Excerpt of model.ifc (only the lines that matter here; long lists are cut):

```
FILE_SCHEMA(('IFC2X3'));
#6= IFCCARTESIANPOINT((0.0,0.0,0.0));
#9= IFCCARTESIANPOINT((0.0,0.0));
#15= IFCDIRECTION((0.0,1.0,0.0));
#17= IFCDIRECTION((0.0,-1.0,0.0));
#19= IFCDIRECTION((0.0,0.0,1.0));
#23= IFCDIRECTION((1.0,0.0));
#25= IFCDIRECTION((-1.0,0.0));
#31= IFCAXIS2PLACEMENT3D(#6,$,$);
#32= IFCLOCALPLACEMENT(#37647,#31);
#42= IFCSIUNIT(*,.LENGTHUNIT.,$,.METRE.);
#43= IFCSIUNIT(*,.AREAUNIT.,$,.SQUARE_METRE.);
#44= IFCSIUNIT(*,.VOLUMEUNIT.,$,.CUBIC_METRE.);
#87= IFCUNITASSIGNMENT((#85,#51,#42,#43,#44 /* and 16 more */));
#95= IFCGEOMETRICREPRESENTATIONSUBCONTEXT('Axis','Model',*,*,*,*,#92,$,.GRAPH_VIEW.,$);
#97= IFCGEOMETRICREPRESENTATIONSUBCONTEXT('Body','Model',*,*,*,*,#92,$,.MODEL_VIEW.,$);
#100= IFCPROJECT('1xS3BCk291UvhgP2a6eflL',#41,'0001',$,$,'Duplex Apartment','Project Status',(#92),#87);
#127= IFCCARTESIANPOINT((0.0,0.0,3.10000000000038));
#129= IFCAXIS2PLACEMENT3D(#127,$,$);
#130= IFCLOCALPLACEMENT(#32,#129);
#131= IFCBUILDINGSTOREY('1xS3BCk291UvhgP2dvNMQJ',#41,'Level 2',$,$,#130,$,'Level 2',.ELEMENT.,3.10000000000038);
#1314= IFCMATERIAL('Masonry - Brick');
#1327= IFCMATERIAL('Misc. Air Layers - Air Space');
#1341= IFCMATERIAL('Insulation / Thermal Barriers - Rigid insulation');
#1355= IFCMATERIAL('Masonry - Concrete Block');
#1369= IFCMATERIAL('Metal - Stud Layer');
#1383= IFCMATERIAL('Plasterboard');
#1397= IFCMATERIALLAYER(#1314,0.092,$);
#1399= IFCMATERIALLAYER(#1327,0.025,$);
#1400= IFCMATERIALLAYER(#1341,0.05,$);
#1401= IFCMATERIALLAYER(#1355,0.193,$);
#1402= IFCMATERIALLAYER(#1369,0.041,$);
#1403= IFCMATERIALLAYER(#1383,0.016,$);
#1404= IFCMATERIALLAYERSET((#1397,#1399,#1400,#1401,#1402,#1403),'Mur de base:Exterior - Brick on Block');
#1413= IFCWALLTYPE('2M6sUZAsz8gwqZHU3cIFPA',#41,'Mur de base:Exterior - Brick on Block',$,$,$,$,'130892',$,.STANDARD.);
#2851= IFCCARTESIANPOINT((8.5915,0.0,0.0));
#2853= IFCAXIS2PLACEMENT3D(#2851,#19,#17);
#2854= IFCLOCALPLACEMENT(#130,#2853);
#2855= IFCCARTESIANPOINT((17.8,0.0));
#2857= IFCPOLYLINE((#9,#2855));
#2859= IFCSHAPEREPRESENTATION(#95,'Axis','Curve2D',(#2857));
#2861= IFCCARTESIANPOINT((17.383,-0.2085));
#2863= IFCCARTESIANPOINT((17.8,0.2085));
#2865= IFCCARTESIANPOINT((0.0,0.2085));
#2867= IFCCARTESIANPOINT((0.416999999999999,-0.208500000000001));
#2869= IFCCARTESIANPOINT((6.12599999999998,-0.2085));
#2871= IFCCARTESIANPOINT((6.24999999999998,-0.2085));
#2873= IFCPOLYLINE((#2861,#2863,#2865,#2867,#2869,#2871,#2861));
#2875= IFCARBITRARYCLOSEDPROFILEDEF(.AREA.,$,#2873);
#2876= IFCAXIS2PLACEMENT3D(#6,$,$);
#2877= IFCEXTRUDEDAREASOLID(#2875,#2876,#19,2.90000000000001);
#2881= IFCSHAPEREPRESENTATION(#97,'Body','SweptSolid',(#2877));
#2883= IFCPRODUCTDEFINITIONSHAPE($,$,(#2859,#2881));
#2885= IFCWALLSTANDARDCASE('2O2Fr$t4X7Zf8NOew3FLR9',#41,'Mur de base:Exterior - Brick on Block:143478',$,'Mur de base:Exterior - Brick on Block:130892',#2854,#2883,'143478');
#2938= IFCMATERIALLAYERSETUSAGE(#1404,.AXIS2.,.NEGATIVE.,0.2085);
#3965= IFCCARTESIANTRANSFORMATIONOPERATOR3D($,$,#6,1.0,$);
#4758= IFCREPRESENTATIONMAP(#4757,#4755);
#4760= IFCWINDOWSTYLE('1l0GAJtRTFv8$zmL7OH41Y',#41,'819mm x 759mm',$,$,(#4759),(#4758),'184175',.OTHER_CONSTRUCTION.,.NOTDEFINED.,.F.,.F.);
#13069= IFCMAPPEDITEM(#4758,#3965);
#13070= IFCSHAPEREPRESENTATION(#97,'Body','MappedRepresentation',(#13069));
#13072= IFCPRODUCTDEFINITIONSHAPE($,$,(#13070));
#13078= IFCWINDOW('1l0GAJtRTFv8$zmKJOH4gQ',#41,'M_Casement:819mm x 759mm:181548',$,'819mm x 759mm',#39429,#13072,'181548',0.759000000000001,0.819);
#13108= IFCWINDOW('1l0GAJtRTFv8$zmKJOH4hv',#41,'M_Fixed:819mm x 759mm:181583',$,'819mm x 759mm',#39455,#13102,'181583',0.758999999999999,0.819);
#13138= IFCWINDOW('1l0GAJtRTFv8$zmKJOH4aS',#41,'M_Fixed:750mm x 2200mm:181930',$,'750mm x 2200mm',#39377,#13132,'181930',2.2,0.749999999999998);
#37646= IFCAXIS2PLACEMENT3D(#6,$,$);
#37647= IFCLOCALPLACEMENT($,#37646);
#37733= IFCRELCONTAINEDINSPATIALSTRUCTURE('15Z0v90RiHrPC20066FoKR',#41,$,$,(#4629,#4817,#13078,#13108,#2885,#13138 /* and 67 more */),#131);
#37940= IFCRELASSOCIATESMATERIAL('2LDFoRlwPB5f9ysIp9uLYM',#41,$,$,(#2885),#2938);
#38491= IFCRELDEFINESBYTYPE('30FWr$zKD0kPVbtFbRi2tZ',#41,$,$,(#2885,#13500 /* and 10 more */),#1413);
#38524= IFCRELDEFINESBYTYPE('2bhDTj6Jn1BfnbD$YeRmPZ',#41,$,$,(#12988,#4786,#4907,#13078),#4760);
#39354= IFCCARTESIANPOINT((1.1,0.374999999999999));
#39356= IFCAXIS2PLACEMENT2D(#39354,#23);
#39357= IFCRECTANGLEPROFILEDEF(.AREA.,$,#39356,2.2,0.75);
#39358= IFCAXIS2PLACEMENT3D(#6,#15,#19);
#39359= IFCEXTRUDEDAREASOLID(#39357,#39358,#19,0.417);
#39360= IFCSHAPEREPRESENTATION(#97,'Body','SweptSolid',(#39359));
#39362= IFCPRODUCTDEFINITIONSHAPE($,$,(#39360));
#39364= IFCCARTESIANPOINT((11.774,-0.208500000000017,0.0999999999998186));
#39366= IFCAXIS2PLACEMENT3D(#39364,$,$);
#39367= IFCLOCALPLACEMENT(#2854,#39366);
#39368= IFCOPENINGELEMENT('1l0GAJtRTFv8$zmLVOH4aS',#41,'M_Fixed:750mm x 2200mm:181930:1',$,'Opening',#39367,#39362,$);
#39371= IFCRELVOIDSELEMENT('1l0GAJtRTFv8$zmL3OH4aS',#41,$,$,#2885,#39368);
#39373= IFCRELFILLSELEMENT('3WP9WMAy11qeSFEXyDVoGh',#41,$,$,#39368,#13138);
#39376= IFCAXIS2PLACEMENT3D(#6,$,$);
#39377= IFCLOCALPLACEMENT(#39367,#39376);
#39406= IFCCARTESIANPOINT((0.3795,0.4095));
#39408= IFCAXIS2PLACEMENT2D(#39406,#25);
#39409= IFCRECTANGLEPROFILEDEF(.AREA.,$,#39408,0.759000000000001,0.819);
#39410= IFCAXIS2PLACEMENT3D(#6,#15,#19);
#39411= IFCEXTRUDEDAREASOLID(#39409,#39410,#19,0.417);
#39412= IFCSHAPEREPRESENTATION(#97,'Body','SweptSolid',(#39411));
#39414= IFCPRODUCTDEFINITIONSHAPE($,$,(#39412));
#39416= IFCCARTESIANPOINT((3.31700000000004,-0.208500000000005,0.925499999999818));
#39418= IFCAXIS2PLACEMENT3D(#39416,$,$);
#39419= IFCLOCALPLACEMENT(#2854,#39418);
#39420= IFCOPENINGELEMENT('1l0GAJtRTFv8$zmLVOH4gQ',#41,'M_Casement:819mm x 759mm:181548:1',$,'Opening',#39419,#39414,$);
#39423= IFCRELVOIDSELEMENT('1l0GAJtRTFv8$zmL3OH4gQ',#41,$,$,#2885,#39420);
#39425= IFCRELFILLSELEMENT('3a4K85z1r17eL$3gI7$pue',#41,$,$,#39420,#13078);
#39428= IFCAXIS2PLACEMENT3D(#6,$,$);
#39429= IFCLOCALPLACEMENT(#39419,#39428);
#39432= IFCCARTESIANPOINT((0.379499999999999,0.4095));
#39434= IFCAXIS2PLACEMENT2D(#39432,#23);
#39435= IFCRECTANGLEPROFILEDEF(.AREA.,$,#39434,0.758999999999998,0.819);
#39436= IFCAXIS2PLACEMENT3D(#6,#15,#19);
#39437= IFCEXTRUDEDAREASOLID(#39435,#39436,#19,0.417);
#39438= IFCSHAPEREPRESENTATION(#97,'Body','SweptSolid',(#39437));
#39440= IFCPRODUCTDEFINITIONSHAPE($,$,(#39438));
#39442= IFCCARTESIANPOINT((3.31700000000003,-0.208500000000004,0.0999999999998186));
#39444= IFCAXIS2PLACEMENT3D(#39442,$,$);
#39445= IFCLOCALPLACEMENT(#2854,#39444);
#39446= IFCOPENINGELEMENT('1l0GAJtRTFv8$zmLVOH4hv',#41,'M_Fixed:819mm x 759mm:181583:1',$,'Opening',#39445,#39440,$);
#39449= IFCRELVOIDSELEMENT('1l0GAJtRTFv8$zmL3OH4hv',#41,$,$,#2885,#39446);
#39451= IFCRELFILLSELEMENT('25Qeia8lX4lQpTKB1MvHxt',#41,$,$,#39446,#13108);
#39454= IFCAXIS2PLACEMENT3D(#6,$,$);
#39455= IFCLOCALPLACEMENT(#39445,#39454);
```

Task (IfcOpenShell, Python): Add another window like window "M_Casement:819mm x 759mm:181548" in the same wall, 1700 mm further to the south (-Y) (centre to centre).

```python
import ifcopenshell
import ifcopenshell.api.feature
import ifcopenshell.api.geometry
import ifcopenshell.api.root
import ifcopenshell.geom
import ifcopenshell.util.element
import ifcopenshell.util.placement
import ifcopenshell.util.shape
import ifcopenshell.util.unit

model = ifcopenshell.open("model.ifc")
unit_scale = ifcopenshell.util.unit.calculate_unit_scale(model)
settings = ifcopenshell.geom.settings()


def volume(element):
    """Net volume in cubic metres, openings subtracted."""
    shape = ifcopenshell.geom.create_shape(settings, element)
    return ifcopenshell.util.shape.get_volume(shape.geometry)


def reuse_history(source, copy):
    """copy_class also copies each property set's owner history, people and application; keep the originals."""
    for rel in copy.IsDefinedBy:
        if rel.is_a("IfcRelDefinesByProperties") and (history := rel.RelatingPropertyDefinition.OwnerHistory):
            rel.RelatingPropertyDefinition.OwnerHistory = source.OwnerHistory
            ifcopenshell.util.element.remove_deep2(model, history)


window = model.by_guid("1l0GAJtRTFv8$zmKJOH4gQ")
opening = window.FillsVoids[0].RelatingOpeningElement
wall = opening.VoidsElements[0].RelatingBuildingElement
before = volume(wall)
shift = ifcopenshell.util.placement.get_local_placement(wall.ObjectPlacement)[:3, 0] * 1.7 / unit_scale

# copy_class copies the void relationship, type, container and properties, but no geometry.
new_opening = ifcopenshell.api.root.copy_class(model, product=opening)
new_opening.Representation = ifcopenshell.util.element.copy_deep(
    model, opening.Representation, exclude=["IfcGeometricRepresentationContext", "IfcRepresentationMap"]
)
new_opening.Name = "M_Casement:819mm x 759mm"
new_window = ifcopenshell.api.root.copy_class(model, product=window)
new_window.Representation = ifcopenshell.util.element.copy_deep(
    model, window.Representation, exclude=["IfcGeometricRepresentationContext", "IfcRepresentationMap"]
)
new_window.Name = "M_Casement:819mm x 759mm"
new_window.Tag = None
reuse_history(window, new_window)
fills = ifcopenshell.api.feature.add_filling(model, opening=new_opening, element=new_window)
fills.OwnerHistory = new_window.OwnerHistory  # required in IFC2X3

for old, new in ((opening, new_opening), (window, new_window)):
    matrix = ifcopenshell.util.placement.get_local_placement(old.ObjectPlacement)
    matrix[:3, 3] += shift
    ifcopenshell.api.geometry.edit_object_placement(model, product=new, matrix=matrix, is_si=False)

after = volume(wall)

print(f"wall volume {before:.3f} -> {after:.3f} m3")

model.write("model_updated.ifc")
```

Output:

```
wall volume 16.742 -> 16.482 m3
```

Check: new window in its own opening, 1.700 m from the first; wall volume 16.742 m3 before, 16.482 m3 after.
